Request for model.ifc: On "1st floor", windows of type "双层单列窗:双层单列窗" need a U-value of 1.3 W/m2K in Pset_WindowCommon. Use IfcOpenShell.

First a look at what the model holds.

```python
import ifcopenshell
import ifcopenshell.util.element

model = ifcopenshell.open("model.ifc")
print(model.schema)
storey = next(s for s in model.by_type("IfcBuildingStorey") if s.Name == "1st floor")
windows = [e for e in ifcopenshell.util.element.get_decomposition(storey) if e.is_a("IfcWindow")]
seen = {}
for e in windows:
    element_type = ifcopenshell.util.element.get_type(e)
    key = (element_type.Name if element_type != e and element_type else None, ifcopenshell.util.element.get_pset(e, "Pset_WindowCommon", "ThermalTransmittance"))
    seen[key] = seen.get(key, 0) + 1
for (name, value), count in sorted(seen.items(), key=str):
    print(count, "x", name, "|", value)
```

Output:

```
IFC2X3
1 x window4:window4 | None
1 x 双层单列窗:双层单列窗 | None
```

```python
import ifcopenshell
import ifcopenshell.api.pset
import ifcopenshell.util.element

model = ifcopenshell.open("model.ifc")

storey = next(s for s in model.by_type("IfcBuildingStorey") if s.Name == "1st floor")
windows = [e for e in ifcopenshell.util.element.get_decomposition(storey) if e.is_a("IfcWindow")]

count = 0
for e in windows:
    element_type = ifcopenshell.util.element.get_type(e)
    if element_type in (None, e) or element_type.Name != "双层单列窗:双层单列窗":
        continue
    # add_pset returns the element's existing set when there is one.
    pset = ifcopenshell.api.pset.add_pset(model, product=e, name="Pset_WindowCommon")
    ifcopenshell.api.pset.edit_pset(model, pset=pset, properties={"ThermalTransmittance": 1.3})
    count += 1

print(count, "windows updated")

model.write("model_updated.ifc")
```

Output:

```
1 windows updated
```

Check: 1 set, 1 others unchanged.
